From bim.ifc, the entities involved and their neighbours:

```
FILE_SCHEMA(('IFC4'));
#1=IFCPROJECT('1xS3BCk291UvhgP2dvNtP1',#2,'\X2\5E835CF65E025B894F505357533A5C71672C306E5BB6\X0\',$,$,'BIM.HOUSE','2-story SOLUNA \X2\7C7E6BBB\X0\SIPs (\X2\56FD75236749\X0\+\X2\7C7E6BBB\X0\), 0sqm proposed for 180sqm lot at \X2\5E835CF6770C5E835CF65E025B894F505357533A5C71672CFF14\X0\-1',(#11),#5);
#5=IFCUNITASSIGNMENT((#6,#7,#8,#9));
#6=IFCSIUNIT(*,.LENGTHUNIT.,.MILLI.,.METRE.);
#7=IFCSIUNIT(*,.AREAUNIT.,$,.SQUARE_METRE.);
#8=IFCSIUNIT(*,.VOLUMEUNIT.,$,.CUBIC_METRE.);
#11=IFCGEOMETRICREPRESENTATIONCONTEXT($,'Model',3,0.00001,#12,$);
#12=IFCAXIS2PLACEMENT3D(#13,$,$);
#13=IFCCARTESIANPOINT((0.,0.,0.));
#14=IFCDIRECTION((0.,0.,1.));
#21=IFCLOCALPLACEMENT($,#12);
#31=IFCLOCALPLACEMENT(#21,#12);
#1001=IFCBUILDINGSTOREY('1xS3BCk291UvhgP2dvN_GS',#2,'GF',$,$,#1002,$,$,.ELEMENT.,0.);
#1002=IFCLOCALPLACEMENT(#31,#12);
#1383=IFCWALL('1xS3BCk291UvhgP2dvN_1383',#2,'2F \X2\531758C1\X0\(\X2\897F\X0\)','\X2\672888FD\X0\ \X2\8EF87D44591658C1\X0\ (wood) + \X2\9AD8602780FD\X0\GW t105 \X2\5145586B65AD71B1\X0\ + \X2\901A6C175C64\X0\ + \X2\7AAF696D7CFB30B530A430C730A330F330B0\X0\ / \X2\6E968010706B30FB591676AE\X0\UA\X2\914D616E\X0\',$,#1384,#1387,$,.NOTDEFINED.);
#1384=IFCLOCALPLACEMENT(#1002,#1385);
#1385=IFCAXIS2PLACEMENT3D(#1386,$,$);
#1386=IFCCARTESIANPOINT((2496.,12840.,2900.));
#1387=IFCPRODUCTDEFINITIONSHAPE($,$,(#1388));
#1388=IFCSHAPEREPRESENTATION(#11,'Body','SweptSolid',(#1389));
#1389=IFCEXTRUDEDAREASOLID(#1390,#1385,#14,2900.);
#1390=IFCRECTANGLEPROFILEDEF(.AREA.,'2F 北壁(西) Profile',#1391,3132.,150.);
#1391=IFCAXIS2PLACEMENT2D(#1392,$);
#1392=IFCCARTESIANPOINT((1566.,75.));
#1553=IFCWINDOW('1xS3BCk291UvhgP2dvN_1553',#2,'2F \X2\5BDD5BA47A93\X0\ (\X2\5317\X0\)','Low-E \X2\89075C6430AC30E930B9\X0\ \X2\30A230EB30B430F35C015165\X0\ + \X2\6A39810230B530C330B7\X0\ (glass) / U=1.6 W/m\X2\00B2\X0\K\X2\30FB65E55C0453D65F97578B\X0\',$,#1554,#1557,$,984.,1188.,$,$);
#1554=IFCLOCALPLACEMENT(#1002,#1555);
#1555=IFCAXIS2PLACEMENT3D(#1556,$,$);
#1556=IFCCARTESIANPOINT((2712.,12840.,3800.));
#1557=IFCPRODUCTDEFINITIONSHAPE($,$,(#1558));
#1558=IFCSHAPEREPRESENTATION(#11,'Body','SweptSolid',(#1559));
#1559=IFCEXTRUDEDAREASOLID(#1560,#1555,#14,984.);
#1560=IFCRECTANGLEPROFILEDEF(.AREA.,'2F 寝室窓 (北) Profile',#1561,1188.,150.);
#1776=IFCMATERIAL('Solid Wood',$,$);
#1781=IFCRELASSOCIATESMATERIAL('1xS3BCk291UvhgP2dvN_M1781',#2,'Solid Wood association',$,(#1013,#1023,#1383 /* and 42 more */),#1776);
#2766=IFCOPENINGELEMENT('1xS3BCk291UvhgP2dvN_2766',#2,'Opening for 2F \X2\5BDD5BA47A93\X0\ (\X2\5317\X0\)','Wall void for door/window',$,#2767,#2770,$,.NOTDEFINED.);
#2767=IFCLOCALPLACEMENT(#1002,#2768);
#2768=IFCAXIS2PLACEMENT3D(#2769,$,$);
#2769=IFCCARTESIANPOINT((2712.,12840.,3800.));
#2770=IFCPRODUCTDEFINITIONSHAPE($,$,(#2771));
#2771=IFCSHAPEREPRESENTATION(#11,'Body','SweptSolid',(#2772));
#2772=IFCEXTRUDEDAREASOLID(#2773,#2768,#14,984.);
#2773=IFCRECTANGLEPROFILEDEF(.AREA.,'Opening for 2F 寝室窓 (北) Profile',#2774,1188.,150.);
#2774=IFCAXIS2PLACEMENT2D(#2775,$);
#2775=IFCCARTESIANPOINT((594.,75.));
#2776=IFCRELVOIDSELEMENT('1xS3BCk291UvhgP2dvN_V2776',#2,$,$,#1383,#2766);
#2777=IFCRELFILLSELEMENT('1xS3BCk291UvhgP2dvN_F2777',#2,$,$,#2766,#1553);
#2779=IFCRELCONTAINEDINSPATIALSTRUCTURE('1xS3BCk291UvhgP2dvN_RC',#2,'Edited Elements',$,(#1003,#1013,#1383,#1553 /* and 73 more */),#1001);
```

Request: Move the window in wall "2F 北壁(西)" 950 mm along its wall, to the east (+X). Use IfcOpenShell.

```python
import ifcopenshell
import ifcopenshell.api.geometry
import ifcopenshell.util.placement
import ifcopenshell.util.unit

model = ifcopenshell.open("bim.ifc")
unit_scale = ifcopenshell.util.unit.calculate_unit_scale(model)

window = model.by_id(1553)
opening = window.FillsVoids[0].RelatingOpeningElement
wall = opening.VoidsElements[0].RelatingBuildingElement

wall_matrix = ifcopenshell.util.placement.get_local_placement(wall.ObjectPlacement)
shift = wall_matrix[:3, 0] * 0.95 / unit_scale
before = ifcopenshell.util.placement.get_local_placement(window.ObjectPlacement)[:3, 3].copy()

# The window is not placed relative to its opening, so move both.
for product in (opening, window):
    matrix = ifcopenshell.util.placement.get_local_placement(product.ObjectPlacement)
    matrix[:3, 3] += shift
    ifcopenshell.api.geometry.edit_object_placement(model, product=product, matrix=matrix, is_si=False)

after = ifcopenshell.util.placement.get_local_placement(window.ObjectPlacement)[:3, 3]
print("window moved by", (after - before).round(3) + 0.0)

model.write("bim-out.ifc")
```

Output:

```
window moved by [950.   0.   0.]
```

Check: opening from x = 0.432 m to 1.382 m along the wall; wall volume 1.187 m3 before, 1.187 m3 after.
